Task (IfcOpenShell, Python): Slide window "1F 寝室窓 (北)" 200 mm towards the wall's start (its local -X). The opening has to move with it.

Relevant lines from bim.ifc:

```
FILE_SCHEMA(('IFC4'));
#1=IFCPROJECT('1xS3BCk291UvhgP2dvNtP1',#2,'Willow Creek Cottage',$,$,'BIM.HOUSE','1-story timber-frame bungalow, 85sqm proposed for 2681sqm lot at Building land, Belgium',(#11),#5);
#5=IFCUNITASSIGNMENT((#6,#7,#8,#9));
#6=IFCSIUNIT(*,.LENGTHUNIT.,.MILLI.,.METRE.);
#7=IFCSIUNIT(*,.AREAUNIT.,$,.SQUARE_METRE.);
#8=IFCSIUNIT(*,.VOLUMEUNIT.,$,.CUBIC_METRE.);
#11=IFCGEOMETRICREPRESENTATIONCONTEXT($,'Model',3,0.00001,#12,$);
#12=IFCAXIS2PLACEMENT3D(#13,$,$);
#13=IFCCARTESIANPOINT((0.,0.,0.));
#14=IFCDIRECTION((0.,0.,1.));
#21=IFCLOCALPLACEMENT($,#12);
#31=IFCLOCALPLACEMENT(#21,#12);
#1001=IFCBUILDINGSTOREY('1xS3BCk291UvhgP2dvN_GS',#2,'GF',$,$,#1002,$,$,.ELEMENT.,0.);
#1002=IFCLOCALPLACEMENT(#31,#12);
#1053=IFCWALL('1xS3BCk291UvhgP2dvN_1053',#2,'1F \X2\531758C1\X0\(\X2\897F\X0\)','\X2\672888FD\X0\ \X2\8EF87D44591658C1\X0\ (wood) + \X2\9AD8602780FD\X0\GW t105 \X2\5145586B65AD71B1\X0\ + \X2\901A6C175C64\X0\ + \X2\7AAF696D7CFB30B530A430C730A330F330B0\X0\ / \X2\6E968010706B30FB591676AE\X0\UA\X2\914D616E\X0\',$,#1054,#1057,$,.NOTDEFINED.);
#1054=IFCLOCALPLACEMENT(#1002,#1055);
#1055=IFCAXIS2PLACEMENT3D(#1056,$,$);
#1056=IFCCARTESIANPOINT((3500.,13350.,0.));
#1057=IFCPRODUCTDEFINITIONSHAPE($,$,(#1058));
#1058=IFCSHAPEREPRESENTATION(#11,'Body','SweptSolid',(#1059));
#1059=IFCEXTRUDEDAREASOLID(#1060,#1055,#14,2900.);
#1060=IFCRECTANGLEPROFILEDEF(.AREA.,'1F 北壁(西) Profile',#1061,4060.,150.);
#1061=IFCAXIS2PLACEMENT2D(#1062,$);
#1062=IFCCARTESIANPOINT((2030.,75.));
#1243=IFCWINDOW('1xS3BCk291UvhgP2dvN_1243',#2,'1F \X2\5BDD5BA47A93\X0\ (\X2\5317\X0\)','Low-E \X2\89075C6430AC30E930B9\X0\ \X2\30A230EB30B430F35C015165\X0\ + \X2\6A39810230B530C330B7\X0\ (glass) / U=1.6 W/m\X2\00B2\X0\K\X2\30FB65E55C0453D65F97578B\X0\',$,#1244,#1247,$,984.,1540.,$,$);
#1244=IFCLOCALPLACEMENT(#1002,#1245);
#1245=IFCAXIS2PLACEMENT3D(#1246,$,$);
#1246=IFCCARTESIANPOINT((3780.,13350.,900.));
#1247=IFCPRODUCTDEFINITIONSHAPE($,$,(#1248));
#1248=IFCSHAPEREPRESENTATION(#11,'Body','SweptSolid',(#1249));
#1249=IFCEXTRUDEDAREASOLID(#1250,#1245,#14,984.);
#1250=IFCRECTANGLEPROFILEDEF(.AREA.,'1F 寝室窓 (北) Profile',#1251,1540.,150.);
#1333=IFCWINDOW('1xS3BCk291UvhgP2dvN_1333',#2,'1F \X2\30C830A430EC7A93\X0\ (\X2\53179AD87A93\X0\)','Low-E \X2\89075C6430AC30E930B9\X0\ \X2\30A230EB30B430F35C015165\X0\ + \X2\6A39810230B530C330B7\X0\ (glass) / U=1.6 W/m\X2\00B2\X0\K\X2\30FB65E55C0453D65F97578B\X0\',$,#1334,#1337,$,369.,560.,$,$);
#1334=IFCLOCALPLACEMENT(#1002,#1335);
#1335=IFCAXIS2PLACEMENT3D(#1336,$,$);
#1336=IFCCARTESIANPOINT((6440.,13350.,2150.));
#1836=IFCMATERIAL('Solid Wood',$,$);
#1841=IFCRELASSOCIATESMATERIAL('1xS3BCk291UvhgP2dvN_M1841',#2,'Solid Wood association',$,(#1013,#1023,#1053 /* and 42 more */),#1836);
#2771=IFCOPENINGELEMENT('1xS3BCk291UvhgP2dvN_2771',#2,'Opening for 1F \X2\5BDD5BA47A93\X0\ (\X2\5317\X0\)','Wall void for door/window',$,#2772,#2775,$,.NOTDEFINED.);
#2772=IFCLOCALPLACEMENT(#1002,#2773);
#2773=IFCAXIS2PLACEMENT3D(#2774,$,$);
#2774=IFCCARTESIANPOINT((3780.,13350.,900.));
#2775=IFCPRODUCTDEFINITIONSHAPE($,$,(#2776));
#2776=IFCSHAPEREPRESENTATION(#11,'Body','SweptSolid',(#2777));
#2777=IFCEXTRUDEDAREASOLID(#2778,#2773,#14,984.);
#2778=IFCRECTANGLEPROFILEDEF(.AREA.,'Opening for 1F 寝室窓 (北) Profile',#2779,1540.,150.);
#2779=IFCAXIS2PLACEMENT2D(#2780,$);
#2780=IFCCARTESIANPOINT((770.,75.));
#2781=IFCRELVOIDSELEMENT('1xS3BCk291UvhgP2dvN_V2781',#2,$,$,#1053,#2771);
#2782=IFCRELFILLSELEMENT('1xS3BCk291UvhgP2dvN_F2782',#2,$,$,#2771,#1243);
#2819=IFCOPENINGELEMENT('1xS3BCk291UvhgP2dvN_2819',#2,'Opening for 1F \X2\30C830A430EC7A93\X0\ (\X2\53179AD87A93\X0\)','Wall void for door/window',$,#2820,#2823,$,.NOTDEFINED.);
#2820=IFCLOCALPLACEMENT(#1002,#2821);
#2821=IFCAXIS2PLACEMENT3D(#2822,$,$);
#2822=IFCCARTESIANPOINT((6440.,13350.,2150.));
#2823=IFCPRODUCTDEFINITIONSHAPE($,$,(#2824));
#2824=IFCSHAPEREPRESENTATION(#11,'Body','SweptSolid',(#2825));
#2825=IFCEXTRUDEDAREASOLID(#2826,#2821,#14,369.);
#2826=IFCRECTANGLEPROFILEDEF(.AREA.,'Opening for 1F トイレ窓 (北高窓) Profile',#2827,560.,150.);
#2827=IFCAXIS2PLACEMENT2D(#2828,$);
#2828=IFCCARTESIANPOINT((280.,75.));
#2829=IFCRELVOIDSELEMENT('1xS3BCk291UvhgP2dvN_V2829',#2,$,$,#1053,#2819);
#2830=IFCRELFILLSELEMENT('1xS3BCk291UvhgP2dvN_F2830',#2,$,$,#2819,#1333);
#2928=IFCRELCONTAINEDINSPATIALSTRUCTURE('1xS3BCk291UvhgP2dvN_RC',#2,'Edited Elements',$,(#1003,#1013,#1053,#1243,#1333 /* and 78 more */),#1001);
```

```python
import ifcopenshell
import ifcopenshell.api.geometry
import ifcopenshell.util.placement
import ifcopenshell.util.unit

model = ifcopenshell.open("bim.ifc")
unit_scale = ifcopenshell.util.unit.calculate_unit_scale(model)

window = model.by_guid("1xS3BCk291UvhgP2dvN_1243")
opening = window.FillsVoids[0].RelatingOpeningElement
wall = opening.VoidsElements[0].RelatingBuildingElement

wall_matrix = ifcopenshell.util.placement.get_local_placement(wall.ObjectPlacement)
shift = wall_matrix[:3, 0] * -0.2 / unit_scale
before = ifcopenshell.util.placement.get_local_placement(window.ObjectPlacement)[:3, 3].copy()

# The window is not placed relative to its opening, so move both.
for product in (opening, window):
    matrix = ifcopenshell.util.placement.get_local_placement(product.ObjectPlacement)
    matrix[:3, 3] += shift
    ifcopenshell.api.geometry.edit_object_placement(model, product=product, matrix=matrix, is_si=False)

after = ifcopenshell.util.placement.get_local_placement(window.ObjectPlacement)[:3, 3]
print("window moved by", (after - before).round(3) + 0.0)

model.write("bim_edited.ifc")
```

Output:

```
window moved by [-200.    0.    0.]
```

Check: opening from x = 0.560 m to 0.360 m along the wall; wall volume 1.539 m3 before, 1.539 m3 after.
